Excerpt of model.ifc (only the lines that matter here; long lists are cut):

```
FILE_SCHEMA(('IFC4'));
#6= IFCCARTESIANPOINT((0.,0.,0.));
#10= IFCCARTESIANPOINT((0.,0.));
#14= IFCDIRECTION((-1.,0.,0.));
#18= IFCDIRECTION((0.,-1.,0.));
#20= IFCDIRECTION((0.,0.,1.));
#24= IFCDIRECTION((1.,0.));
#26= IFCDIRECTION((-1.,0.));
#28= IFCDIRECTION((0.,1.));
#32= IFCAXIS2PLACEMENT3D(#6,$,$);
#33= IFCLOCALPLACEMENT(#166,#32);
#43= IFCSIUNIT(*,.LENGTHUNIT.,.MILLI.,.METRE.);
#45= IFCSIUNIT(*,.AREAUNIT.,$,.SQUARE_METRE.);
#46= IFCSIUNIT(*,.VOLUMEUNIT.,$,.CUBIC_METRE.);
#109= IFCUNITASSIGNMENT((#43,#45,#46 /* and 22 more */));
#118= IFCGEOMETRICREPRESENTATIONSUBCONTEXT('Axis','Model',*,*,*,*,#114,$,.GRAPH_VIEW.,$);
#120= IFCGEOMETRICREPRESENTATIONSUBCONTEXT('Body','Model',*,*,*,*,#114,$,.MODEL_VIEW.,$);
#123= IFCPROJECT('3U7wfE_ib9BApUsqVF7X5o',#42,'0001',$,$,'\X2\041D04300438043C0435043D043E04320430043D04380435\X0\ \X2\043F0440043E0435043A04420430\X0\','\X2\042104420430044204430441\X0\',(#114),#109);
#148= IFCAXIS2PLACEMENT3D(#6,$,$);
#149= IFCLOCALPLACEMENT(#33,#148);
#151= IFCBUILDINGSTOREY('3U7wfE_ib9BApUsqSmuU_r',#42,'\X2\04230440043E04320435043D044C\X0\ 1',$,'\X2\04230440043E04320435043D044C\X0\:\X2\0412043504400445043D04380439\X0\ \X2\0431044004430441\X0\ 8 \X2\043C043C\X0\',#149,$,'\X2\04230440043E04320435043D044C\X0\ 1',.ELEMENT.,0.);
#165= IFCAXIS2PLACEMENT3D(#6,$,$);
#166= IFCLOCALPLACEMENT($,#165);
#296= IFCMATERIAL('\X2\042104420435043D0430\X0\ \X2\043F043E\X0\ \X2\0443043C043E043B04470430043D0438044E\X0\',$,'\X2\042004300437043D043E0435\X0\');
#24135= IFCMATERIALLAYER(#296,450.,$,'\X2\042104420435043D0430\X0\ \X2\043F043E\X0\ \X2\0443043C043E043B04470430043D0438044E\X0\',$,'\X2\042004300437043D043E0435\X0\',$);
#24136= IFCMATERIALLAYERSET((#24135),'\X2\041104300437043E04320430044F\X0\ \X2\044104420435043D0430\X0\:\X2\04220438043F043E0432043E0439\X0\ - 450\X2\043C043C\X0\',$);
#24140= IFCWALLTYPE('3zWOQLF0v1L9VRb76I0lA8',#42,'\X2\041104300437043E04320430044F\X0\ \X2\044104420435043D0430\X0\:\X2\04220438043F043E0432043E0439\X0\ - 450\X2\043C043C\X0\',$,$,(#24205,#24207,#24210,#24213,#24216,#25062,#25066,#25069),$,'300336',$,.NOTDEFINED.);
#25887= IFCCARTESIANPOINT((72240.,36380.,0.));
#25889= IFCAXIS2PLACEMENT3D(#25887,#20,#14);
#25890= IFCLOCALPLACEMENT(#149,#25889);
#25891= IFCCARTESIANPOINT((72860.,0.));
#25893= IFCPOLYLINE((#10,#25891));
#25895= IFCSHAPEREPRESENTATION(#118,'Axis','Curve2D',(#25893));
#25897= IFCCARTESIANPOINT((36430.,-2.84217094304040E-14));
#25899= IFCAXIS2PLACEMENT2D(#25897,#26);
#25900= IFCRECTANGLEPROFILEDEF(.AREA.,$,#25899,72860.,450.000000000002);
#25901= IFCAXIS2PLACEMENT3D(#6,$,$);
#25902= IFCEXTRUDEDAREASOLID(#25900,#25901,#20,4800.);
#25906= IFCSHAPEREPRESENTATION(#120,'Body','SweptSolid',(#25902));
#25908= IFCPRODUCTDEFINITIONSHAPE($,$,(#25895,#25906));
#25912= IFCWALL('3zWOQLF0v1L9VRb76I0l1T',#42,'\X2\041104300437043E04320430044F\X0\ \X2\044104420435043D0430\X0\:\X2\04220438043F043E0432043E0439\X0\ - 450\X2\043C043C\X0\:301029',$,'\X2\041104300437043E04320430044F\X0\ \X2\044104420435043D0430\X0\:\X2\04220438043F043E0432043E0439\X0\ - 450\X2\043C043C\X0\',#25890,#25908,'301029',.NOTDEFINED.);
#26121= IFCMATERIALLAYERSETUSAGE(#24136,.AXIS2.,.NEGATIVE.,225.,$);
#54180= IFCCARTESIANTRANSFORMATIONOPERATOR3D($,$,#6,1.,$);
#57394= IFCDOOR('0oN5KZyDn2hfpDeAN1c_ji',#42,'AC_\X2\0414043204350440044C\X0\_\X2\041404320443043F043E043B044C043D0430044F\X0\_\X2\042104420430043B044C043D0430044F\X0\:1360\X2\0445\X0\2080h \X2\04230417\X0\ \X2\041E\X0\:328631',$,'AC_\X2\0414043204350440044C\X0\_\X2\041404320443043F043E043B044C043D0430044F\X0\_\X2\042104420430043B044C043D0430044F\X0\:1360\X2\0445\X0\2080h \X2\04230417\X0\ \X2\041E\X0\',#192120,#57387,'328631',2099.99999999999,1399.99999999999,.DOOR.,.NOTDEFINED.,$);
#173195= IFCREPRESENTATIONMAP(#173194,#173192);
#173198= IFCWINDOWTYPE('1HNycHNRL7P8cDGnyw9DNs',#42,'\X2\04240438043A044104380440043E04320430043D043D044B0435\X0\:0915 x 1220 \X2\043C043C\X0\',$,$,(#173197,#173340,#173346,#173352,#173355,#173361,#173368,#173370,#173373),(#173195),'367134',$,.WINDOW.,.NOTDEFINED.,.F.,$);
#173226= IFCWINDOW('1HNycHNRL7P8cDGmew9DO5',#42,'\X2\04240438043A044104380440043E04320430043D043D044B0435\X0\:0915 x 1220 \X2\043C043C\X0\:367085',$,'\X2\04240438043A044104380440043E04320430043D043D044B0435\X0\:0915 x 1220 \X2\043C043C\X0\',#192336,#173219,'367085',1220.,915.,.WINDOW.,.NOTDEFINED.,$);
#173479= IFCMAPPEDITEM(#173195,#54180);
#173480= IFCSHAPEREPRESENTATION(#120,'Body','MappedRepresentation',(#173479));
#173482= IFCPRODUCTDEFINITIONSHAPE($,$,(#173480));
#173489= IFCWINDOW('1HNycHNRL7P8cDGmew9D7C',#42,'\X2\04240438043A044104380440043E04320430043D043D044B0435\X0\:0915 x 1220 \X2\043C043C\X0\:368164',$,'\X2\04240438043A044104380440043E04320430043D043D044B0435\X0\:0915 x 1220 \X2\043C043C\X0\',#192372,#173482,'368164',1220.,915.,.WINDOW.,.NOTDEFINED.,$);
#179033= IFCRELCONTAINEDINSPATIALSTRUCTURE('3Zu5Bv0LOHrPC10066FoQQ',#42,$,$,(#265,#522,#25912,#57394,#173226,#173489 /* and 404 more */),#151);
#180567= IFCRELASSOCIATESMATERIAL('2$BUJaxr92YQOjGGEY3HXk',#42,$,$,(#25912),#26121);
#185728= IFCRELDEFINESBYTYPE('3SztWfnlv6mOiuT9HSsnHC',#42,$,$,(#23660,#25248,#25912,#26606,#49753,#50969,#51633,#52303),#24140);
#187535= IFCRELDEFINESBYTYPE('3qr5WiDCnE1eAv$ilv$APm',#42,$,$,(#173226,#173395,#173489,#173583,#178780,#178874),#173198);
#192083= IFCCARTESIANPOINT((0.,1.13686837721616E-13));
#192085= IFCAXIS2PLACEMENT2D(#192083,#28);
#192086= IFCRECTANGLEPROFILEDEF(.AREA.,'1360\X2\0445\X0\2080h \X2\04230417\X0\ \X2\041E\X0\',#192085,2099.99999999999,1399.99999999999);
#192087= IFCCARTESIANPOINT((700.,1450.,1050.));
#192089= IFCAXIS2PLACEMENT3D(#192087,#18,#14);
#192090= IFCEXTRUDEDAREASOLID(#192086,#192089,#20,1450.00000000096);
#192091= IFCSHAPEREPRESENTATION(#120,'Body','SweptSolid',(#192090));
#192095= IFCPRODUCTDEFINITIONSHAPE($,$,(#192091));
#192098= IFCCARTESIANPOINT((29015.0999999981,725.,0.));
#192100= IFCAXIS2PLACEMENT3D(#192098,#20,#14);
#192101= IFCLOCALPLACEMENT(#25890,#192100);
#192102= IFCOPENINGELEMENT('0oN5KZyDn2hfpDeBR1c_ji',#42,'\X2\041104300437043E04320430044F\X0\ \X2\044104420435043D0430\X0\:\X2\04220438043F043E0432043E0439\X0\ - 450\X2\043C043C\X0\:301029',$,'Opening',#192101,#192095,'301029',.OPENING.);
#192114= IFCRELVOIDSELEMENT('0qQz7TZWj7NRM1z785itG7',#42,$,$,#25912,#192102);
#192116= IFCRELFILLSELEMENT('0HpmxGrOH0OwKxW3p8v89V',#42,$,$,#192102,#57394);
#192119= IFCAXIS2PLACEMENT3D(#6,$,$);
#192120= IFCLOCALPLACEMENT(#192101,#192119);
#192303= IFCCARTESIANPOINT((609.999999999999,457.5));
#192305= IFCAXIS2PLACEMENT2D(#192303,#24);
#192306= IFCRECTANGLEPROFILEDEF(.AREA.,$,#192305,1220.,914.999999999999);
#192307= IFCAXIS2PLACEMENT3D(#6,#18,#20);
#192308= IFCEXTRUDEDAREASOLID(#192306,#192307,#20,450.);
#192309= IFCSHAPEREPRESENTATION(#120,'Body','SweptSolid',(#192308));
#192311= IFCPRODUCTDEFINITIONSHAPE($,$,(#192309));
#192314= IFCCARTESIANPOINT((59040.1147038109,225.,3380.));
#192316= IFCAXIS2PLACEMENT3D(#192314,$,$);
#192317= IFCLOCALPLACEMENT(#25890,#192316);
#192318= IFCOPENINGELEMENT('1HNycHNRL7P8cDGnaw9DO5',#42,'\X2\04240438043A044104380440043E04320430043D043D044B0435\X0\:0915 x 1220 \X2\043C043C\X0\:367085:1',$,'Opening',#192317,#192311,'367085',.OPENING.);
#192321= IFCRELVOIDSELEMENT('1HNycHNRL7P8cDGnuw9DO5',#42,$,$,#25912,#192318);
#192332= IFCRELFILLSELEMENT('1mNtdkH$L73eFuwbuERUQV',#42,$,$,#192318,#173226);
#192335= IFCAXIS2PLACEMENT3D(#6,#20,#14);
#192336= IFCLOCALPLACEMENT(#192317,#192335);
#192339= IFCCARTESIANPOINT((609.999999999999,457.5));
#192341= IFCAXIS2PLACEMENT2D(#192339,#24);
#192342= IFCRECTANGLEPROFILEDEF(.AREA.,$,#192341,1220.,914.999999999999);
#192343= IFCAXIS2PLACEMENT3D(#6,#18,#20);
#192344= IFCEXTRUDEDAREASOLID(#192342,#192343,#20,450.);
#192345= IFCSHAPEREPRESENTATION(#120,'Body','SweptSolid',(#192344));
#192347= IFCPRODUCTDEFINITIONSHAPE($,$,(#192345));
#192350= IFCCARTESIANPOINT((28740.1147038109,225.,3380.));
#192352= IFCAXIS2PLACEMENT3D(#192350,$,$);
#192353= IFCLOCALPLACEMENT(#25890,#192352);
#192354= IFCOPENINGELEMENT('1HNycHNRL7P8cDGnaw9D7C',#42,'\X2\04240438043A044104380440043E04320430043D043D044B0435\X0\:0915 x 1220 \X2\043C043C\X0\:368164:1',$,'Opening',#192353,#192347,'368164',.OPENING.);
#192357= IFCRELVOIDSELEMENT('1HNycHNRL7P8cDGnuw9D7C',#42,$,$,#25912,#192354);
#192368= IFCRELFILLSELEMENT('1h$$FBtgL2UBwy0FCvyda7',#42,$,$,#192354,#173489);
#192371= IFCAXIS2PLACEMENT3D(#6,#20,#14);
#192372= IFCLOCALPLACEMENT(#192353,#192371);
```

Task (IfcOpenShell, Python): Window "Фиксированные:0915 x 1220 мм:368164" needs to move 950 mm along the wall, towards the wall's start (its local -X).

```python
import ifcopenshell
import ifcopenshell.api.geometry
import ifcopenshell.util.placement

model = ifcopenshell.open("model.ifc")

window = model.by_guid("1HNycHNRL7P8cDGmew9D7C")
opening = window.FillsVoids[0].RelatingOpeningElement
wall = opening.VoidsElements[0].RelatingBuildingElement

wall_matrix = ifcopenshell.util.placement.get_local_placement(wall.ObjectPlacement)
shift = wall_matrix[:3, 0] * -950.0
before = ifcopenshell.util.placement.get_local_placement(window.ObjectPlacement)[:3, 3].copy()

# The window is placed relative to its opening, so it follows when the opening moves.
matrix = ifcopenshell.util.placement.get_local_placement(opening.ObjectPlacement)
matrix[:3, 3] += shift
ifcopenshell.api.geometry.edit_object_placement(
    model, product=opening, matrix=matrix, is_si=False, should_transform_children=True
)

after = ifcopenshell.util.placement.get_local_placement(window.ObjectPlacement)[:3, 3]
print("window moved by", (after - before).round(3) + 0.0)

model.write("model_rev.ifc")
```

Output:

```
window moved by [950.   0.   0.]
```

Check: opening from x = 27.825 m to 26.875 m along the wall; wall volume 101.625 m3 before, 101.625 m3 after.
